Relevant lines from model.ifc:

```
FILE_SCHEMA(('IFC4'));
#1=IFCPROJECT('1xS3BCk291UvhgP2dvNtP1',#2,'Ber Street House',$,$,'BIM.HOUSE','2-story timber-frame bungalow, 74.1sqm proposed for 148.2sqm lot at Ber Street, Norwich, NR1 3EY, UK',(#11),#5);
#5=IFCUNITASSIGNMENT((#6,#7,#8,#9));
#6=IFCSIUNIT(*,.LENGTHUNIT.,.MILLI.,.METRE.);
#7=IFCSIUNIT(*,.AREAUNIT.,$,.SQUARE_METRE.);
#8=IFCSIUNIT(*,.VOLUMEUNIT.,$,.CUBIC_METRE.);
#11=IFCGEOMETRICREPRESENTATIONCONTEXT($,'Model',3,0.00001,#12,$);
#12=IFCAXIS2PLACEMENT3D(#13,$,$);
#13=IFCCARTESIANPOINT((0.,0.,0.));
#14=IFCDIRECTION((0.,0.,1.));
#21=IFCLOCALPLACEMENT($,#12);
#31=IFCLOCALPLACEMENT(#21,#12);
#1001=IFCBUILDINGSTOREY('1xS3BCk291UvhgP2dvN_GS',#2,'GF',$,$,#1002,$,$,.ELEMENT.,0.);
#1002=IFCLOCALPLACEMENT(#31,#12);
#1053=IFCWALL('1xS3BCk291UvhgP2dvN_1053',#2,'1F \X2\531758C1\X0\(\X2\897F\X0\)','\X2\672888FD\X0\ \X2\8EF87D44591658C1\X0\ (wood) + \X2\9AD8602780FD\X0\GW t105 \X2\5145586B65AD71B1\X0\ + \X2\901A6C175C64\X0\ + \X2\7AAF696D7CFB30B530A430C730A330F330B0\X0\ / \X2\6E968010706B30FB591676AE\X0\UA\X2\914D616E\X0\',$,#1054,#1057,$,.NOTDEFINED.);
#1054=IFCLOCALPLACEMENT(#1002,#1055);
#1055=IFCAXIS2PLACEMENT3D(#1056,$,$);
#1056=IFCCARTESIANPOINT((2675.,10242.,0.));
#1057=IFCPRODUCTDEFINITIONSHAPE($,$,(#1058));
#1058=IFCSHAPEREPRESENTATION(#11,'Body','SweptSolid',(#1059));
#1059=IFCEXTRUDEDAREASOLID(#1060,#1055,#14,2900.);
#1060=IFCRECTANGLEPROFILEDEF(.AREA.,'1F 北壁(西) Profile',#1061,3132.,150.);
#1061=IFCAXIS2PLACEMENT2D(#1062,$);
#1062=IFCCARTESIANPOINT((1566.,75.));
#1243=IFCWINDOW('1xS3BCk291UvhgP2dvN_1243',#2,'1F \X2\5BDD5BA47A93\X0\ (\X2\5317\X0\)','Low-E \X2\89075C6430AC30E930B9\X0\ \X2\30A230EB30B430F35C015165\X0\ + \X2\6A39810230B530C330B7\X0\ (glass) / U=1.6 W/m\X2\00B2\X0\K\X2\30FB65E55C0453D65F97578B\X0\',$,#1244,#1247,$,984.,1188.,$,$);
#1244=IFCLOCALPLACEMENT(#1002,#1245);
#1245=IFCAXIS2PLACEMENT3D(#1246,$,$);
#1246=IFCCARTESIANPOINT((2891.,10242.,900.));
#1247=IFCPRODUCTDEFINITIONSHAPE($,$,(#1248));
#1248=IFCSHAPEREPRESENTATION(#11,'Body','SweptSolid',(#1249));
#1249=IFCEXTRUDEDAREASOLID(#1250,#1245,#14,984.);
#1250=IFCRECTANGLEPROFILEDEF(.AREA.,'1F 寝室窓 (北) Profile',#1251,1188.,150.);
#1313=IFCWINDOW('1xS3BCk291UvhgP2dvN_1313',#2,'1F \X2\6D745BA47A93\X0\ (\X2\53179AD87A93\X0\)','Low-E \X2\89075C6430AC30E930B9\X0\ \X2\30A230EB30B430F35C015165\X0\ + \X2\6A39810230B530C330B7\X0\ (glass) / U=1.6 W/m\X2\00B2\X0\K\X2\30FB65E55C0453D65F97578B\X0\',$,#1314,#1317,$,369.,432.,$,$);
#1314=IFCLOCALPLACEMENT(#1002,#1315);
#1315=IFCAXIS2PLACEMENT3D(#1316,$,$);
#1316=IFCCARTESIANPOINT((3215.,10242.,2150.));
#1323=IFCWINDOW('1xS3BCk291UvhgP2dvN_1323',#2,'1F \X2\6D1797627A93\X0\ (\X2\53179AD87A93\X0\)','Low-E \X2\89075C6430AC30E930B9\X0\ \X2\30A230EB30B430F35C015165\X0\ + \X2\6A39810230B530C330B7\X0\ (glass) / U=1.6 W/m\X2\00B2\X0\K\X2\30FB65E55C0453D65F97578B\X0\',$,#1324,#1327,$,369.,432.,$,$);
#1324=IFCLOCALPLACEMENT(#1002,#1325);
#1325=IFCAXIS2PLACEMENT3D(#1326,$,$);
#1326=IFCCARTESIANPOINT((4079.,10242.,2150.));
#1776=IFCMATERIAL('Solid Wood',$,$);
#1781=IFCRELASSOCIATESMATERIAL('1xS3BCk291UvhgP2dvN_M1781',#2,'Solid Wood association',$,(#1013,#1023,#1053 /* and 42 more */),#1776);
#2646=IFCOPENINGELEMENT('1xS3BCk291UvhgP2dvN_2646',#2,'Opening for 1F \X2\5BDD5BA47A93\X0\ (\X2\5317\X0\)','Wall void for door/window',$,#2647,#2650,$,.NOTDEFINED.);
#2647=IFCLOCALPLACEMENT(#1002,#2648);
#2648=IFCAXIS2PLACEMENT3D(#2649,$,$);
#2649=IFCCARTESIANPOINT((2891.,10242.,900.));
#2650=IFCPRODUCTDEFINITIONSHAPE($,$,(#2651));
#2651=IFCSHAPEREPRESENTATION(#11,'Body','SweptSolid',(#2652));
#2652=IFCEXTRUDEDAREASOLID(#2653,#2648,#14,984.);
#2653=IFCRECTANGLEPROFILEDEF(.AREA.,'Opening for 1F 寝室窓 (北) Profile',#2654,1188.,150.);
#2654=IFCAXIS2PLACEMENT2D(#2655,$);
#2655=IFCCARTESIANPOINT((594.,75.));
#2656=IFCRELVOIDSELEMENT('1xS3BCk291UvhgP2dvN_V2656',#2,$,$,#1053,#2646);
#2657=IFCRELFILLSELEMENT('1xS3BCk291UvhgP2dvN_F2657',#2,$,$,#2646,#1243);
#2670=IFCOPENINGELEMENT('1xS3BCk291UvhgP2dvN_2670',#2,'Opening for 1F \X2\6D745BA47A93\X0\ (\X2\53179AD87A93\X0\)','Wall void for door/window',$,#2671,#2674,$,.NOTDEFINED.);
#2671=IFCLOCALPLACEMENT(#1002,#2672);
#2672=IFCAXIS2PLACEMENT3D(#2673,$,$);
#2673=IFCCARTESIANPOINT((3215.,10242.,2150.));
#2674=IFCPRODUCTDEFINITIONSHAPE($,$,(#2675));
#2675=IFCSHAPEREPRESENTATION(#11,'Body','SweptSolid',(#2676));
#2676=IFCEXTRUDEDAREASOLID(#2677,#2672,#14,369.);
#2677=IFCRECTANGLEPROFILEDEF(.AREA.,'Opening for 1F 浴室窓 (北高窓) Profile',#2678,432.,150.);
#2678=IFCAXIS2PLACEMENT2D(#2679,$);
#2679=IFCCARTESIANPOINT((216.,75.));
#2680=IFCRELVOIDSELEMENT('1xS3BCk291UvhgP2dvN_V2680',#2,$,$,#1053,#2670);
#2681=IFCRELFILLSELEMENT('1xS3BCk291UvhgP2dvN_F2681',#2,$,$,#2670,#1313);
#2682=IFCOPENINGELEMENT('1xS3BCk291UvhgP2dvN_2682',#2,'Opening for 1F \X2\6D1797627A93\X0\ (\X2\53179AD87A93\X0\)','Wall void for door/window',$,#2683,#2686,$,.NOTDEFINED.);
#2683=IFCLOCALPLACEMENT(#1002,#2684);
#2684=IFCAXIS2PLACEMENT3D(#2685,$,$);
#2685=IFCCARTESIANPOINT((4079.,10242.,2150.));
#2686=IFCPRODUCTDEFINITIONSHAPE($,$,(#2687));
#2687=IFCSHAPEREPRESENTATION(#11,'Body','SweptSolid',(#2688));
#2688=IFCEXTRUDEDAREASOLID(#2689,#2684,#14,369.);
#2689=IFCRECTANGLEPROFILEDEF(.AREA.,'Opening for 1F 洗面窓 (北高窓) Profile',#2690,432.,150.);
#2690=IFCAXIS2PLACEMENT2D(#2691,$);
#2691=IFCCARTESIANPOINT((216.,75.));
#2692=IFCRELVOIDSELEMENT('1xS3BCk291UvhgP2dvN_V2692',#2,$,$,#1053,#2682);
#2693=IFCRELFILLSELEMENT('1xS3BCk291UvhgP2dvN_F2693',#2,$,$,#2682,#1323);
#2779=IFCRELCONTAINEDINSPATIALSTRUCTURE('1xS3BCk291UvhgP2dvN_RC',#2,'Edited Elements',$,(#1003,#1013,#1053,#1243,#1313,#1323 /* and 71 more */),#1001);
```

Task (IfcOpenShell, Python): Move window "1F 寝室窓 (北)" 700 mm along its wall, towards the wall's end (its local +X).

```python
import ifcopenshell
import ifcopenshell.api.geometry
import ifcopenshell.util.placement

model = ifcopenshell.open("model.ifc")

window = model.by_id(1243)
opening = window.FillsVoids[0].RelatingOpeningElement
wall = opening.VoidsElements[0].RelatingBuildingElement

wall_matrix = ifcopenshell.util.placement.get_local_placement(wall.ObjectPlacement)
shift = wall_matrix[:3, 0] * 700.0
before = ifcopenshell.util.placement.get_local_placement(window.ObjectPlacement)[:3, 3].copy()

# The window is not placed relative to its opening, so move both.
for product in (opening, window):
    matrix = ifcopenshell.util.placement.get_local_placement(product.ObjectPlacement)
    matrix[:3, 3] += shift
    ifcopenshell.api.geometry.edit_object_placement(model, product=product, matrix=matrix, is_si=False)

after = ifcopenshell.util.placement.get_local_placement(window.ObjectPlacement)[:3, 3]
print("window moved by", (after - before).round(3) + 0.0)

model.write("model-out.ifc")
```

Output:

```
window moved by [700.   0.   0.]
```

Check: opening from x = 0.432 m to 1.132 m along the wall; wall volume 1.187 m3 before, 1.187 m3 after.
